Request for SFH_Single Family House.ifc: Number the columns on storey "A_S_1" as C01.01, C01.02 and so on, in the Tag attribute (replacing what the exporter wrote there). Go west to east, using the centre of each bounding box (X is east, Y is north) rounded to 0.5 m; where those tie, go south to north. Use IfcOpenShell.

First a look at what the model holds.

```python
import ifcopenshell
import ifcopenshell.util.element
import ifcopenshell.util.placement

model = ifcopenshell.open("SFH_Single Family House.ifc")
print(model.schema)
storey = next(s for s in model.by_type("IfcBuildingStorey") if s.Name == "A_S_1")
columns = [e for e in ifcopenshell.util.element.get_decomposition(storey) if e.is_a("IfcColumn")]
for e in sorted(columns, key=lambda e: e.id()):
    origin = ifcopenshell.util.placement.get_local_placement(e.ObjectPlacement)[:3, 3]
    print(e.id(), e.Tag, e.Name, origin.round(2) + 0.0, sep=" | ")
```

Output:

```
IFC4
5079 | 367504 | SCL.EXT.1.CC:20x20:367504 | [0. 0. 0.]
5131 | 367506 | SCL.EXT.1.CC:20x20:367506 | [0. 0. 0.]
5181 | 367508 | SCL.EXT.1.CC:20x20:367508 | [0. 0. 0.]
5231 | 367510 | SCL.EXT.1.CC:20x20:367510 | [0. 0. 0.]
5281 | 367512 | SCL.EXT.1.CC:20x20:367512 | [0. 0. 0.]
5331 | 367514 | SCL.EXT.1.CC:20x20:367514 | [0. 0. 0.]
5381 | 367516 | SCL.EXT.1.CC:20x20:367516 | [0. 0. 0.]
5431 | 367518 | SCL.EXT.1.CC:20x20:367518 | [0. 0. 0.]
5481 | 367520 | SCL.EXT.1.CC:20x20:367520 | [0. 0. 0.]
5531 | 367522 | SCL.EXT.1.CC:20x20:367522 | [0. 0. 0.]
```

```python
import ifcopenshell
import ifcopenshell.geom
import ifcopenshell.util.element
import ifcopenshell.util.shape

model = ifcopenshell.open("SFH_Single Family House.ifc")
settings = ifcopenshell.geom.settings()
settings.set("use-world-coords", True)


def centre(element):
    shape = ifcopenshell.geom.create_shape(settings, element)
    return ifcopenshell.util.shape.get_bbox_centroid(shape.geometry)


storey = next(s for s in model.by_type("IfcBuildingStorey") if s.Name == "A_S_1")
columns = [e for e in ifcopenshell.util.element.get_decomposition(storey) if e.is_a("IfcColumn")]

# Insertion points can sit at a corner or the storey origin, so sort by the geometry (in metres).
centres = {e: centre(e) for e in columns}
columns.sort(key=lambda e: (round(centres[e][0] / 0.5), centres[e][1]))

for i, e in enumerate(columns, start=1):
    number = f"C01.{i:02d}"
    e.Tag = number
    print(e.id(), number)

model.write("SFH_Single Family House_edited.ifc")
```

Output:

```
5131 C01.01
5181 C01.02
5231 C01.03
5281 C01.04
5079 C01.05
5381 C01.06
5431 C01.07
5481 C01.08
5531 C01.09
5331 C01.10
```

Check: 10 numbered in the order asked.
